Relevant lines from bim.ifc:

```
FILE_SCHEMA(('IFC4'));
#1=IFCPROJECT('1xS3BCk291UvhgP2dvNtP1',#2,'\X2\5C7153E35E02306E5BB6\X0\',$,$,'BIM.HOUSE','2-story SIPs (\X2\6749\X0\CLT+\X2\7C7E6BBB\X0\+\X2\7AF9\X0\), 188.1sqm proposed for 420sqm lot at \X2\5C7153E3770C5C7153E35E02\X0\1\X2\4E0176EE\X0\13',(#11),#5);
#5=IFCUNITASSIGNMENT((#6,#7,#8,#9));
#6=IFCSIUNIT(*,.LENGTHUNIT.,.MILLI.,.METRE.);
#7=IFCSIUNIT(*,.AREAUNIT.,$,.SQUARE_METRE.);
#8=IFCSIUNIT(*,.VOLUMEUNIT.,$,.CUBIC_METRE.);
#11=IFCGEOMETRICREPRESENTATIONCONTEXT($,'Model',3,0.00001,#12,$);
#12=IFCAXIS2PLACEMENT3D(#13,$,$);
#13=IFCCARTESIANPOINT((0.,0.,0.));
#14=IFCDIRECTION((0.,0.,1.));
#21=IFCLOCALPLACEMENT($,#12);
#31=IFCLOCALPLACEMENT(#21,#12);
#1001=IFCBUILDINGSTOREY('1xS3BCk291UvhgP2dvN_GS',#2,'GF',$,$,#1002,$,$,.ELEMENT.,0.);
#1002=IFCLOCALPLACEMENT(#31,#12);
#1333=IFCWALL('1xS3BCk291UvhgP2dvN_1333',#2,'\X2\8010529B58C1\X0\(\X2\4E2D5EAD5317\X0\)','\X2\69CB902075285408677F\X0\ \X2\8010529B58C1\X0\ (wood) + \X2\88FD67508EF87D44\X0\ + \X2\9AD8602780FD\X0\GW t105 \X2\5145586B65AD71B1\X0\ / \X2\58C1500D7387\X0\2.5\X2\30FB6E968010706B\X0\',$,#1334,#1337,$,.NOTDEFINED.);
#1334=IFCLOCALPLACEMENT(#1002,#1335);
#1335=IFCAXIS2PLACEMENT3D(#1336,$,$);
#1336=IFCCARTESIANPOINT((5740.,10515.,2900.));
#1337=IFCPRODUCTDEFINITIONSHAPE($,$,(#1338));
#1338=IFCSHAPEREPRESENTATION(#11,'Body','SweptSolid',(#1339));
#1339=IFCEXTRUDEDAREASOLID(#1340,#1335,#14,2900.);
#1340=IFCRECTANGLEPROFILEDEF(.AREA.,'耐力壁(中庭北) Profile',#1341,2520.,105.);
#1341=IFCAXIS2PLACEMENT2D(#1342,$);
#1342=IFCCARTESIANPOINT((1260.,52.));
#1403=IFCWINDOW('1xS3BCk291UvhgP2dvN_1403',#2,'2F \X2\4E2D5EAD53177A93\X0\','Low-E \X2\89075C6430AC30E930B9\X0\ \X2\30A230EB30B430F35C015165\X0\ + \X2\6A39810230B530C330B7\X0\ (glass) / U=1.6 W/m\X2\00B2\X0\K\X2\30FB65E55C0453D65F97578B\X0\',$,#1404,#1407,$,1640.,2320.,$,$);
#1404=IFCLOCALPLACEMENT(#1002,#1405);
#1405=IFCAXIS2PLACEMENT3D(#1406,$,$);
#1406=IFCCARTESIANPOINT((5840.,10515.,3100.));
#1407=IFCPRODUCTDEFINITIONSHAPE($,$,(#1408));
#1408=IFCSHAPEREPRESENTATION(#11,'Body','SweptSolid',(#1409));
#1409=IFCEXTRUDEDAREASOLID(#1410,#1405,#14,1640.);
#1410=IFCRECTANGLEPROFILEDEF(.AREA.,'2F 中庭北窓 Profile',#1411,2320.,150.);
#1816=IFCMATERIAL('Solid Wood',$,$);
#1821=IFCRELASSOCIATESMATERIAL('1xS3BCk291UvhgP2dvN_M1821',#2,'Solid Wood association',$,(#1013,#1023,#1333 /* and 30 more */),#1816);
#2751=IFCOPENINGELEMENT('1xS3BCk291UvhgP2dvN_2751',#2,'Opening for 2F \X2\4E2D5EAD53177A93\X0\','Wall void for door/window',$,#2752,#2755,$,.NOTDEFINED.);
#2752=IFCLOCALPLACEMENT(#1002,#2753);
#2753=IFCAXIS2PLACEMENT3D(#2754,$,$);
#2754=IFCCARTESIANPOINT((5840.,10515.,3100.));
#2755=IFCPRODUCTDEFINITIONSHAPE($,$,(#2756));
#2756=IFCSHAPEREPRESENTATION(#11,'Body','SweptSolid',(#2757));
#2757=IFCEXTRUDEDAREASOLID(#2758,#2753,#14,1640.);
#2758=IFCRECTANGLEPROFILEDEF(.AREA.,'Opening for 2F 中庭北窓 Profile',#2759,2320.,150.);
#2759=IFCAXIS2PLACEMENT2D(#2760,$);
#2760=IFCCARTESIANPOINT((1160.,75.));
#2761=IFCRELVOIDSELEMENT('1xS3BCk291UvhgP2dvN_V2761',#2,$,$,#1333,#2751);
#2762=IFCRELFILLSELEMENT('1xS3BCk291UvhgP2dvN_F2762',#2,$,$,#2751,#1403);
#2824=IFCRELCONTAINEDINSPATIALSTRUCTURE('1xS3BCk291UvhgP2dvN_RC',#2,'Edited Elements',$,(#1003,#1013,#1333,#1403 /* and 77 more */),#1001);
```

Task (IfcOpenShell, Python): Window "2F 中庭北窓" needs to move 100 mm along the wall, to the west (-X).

```python
import ifcopenshell
import ifcopenshell.api.geometry
import ifcopenshell.util.placement

model = ifcopenshell.open("bim.ifc")

window = model.by_guid("1xS3BCk291UvhgP2dvN_1403")
opening = window.FillsVoids[0].RelatingOpeningElement
wall = opening.VoidsElements[0].RelatingBuildingElement

wall_matrix = ifcopenshell.util.placement.get_local_placement(wall.ObjectPlacement)
shift = wall_matrix[:3, 0] * -100.0
before = ifcopenshell.util.placement.get_local_placement(window.ObjectPlacement)[:3, 3].copy()

# The window is not placed relative to its opening, so move both.
for product in (opening, window):
    matrix = ifcopenshell.util.placement.get_local_placement(product.ObjectPlacement)
    matrix[:3, 3] += shift
    ifcopenshell.api.geometry.edit_object_placement(model, product=product, matrix=matrix, is_si=False)

after = ifcopenshell.util.placement.get_local_placement(window.ObjectPlacement)[:3, 3]
print("window moved by", (after - before).round(3) + 0.0)

model.write("bim_updated.ifc")
```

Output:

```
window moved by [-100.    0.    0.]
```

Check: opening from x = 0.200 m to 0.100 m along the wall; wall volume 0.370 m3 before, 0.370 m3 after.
